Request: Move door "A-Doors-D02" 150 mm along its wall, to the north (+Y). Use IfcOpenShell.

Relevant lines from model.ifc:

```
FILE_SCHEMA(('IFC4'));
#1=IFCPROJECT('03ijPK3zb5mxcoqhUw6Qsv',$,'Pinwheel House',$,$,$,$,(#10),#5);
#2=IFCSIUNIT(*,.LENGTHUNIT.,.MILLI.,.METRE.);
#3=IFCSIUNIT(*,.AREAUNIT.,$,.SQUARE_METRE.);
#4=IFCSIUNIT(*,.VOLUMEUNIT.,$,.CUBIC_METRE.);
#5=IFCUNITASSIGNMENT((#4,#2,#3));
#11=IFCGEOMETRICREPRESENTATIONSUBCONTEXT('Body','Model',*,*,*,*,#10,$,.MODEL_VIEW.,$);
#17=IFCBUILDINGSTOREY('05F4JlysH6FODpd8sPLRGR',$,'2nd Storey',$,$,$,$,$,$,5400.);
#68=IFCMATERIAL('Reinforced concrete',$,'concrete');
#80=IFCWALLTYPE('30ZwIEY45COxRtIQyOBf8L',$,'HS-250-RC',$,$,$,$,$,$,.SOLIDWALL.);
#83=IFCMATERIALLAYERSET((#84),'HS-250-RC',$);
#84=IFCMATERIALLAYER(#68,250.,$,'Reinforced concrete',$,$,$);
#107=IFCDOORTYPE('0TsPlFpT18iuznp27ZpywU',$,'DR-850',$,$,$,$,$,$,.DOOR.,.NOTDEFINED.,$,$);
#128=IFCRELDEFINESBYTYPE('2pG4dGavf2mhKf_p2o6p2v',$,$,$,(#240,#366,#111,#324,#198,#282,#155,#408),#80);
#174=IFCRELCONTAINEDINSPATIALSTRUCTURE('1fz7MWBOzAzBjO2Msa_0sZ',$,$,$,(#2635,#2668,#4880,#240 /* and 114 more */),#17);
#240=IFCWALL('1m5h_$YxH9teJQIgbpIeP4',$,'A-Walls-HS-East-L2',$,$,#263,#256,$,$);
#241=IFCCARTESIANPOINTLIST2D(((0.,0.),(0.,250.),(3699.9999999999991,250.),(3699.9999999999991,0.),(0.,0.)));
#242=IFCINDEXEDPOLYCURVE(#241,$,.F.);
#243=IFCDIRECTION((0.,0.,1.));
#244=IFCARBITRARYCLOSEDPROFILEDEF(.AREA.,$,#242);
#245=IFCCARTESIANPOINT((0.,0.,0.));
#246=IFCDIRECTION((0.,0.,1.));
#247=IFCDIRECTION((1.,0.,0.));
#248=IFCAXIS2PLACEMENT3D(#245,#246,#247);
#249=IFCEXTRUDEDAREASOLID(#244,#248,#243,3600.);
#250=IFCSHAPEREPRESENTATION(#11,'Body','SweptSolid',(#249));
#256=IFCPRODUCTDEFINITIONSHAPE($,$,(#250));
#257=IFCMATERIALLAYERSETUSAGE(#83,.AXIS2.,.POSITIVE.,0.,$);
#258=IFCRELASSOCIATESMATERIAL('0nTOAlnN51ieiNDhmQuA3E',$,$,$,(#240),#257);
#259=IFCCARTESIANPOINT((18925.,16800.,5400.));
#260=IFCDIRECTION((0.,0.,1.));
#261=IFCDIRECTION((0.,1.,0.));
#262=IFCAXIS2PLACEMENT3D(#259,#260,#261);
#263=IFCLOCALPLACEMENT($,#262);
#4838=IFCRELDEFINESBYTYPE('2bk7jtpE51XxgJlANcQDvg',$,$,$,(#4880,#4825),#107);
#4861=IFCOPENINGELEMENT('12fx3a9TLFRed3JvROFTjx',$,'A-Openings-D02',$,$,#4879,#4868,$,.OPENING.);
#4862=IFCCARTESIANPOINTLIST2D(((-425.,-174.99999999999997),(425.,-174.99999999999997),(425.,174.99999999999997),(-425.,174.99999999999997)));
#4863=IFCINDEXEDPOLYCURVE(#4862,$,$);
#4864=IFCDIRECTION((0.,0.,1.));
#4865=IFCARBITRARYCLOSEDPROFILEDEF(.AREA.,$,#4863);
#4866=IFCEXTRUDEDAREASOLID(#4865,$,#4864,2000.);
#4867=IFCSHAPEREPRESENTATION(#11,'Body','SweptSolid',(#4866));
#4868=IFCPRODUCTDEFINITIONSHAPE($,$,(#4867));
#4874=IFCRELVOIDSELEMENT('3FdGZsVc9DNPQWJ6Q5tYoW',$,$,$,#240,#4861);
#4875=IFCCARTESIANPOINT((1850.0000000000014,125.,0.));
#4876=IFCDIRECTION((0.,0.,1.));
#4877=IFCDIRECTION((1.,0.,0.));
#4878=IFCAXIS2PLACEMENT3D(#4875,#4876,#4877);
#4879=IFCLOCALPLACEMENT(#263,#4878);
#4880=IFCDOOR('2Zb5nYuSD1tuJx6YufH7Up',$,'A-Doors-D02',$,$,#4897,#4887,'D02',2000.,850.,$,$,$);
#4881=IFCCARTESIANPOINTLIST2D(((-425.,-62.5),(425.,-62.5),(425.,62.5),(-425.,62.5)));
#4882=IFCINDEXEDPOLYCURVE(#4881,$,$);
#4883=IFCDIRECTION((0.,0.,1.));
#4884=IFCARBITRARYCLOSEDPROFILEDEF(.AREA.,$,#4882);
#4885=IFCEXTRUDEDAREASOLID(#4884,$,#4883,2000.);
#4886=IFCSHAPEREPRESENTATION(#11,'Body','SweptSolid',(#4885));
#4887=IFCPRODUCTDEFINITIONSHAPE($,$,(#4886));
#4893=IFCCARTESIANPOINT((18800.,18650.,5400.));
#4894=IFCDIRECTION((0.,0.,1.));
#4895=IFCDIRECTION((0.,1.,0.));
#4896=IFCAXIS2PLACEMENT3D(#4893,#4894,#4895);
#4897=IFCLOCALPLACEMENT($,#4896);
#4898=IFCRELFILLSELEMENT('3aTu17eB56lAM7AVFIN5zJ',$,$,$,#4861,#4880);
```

```python
import ifcopenshell
import ifcopenshell.api.geometry
import ifcopenshell.util.placement

model = ifcopenshell.open("model.ifc")

door = model.by_guid("2Zb5nYuSD1tuJx6YufH7Up")
opening = door.FillsVoids[0].RelatingOpeningElement
wall = opening.VoidsElements[0].RelatingBuildingElement

wall_matrix = ifcopenshell.util.placement.get_local_placement(wall.ObjectPlacement)
shift = wall_matrix[:3, 0] * 150.0
before = ifcopenshell.util.placement.get_local_placement(door.ObjectPlacement)[:3, 3].copy()

# The door is not placed relative to its opening, so move both.
for product in (opening, door):
    matrix = ifcopenshell.util.placement.get_local_placement(product.ObjectPlacement)
    matrix[:3, 3] += shift
    ifcopenshell.api.geometry.edit_object_placement(model, product=product, matrix=matrix, is_si=False)

after = ifcopenshell.util.placement.get_local_placement(door.ObjectPlacement)[:3, 3]
print("door moved by", (after - before).round(3) + 0.0)

model.write("model_updated.ifc")
```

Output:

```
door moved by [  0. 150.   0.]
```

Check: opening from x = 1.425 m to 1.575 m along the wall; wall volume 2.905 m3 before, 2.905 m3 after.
